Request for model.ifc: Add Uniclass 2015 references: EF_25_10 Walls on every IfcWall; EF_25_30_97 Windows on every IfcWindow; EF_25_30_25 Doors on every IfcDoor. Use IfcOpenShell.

First a look at what the model holds.

```python
import ifcopenshell

model = ifcopenshell.open("model.ifc")
print(model.schema)
print("classifications:", [c.Name for c in model.by_type("IfcClassification")])
for ifc_class in ("IfcDoor", "IfcRoof", "IfcStair", "IfcWall", "IfcWindow"):
    print(ifc_class, len(model.by_type(ifc_class)))
```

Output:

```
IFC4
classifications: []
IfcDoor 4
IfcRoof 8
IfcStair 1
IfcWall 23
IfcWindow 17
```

```python
import ifcopenshell
import ifcopenshell.api.classification

model = ifcopenshell.open("model.ifc")

system = ifcopenshell.api.classification.add_classification(model, classification="Uniclass 2015")

codes = {
    "IfcWall": ("EF_25_10", "Walls"),
    "IfcWindow": ("EF_25_30_97", "Windows"),
    "IfcDoor": ("EF_25_30_25", "Doors"),
}
for ifc_class, (code, name) in codes.items():
    products = model.by_type(ifc_class)
    ifcopenshell.api.classification.add_reference(
        model, products=products, classification=system, identification=code, name=name
    )
    print(code, len(products))

model.write("model_rev.ifc")
```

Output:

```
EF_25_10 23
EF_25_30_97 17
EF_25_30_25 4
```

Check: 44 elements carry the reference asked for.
